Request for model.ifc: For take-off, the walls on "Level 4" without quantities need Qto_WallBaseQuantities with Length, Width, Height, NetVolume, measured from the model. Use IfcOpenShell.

First a look at what the model holds.

```python
import ifcopenshell
import ifcopenshell.util.element
import ifcopenshell.util.unit

model = ifcopenshell.open("model.ifc")
print(model.schema)
for unit_type in ("LENGTHUNIT", "AREAUNIT", "VOLUMEUNIT"):
    print(unit_type, ifcopenshell.util.unit.calculate_unit_scale(model, unit_type))
storey = next(s for s in model.by_type("IfcBuildingStorey") if s.Name == "Level 4")
walls = [e for e in ifcopenshell.util.element.get_decomposition(storey) if e.is_a("IfcWall")]
for e in sorted(walls, key=lambda e: e.id()):
    print(e.id(), e.is_a(), e.Name, list(ifcopenshell.util.element.get_psets(e, qtos_only=True)), sep=" | ")
```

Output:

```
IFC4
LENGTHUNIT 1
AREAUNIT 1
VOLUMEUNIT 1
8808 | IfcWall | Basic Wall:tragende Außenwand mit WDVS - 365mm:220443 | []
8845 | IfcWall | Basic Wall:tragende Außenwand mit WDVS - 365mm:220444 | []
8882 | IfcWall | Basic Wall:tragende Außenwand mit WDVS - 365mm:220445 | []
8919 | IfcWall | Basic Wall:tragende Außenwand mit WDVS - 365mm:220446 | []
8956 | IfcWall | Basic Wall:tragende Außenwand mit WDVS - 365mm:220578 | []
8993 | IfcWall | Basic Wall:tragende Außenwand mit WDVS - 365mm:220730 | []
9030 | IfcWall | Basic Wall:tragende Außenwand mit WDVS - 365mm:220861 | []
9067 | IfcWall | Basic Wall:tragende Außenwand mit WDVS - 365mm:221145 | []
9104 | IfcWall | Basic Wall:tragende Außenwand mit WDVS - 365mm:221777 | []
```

```python
import ifcopenshell
import ifcopenshell.api.pset
import ifcopenshell.geom
import ifcopenshell.util.element
import ifcopenshell.util.shape
import ifcopenshell.util.unit

model = ifcopenshell.open("model.ifc")
unit_scale = ifcopenshell.util.unit.calculate_unit_scale(model)
volume_scale = ifcopenshell.util.unit.calculate_unit_scale(model, "VOLUMEUNIT")
settings = ifcopenshell.geom.settings()

storey = next(s for s in model.by_type("IfcBuildingStorey") if s.Name == "Level 4")
walls = [e for e in ifcopenshell.util.element.get_decomposition(storey) if e.is_a("IfcWall")]

for e in sorted(walls, key=lambda e: e.id()):
    if ifcopenshell.util.element.get_psets(e, qtos_only=True, should_inherit=False):
        continue
    # Geometry comes back in metres, in the element's own axes.
    shape = ifcopenshell.geom.create_shape(settings, e)
    values = {
        "Length": ifcopenshell.util.shape.get_x(shape.geometry) / unit_scale,
        "Width": ifcopenshell.util.shape.get_y(shape.geometry) / unit_scale,
        "Height": ifcopenshell.util.shape.get_z(shape.geometry) / unit_scale,
        "NetVolume": ifcopenshell.util.shape.get_volume(shape.geometry) / volume_scale,
    }
    qto = ifcopenshell.api.pset.add_qto(model, product=e, name="Qto_WallBaseQuantities")
    ifcopenshell.api.pset.edit_qto(model, qto=qto, properties=values)
    print(e.id(), {k: round(v, 3) for k, v in values.items()})

model.write("model_updated.ifc")
```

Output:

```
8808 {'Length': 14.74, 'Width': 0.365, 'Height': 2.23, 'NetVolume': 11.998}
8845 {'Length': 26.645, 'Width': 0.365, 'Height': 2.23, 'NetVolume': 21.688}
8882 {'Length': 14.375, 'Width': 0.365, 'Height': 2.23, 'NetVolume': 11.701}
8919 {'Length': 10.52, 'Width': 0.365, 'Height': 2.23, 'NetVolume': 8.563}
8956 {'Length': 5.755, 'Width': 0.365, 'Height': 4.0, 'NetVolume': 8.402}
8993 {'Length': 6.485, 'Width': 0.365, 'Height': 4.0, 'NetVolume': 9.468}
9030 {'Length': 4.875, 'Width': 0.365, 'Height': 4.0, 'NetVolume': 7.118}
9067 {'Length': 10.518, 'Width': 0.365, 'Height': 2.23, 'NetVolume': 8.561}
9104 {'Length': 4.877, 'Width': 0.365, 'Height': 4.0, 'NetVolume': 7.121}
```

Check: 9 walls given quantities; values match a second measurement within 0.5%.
